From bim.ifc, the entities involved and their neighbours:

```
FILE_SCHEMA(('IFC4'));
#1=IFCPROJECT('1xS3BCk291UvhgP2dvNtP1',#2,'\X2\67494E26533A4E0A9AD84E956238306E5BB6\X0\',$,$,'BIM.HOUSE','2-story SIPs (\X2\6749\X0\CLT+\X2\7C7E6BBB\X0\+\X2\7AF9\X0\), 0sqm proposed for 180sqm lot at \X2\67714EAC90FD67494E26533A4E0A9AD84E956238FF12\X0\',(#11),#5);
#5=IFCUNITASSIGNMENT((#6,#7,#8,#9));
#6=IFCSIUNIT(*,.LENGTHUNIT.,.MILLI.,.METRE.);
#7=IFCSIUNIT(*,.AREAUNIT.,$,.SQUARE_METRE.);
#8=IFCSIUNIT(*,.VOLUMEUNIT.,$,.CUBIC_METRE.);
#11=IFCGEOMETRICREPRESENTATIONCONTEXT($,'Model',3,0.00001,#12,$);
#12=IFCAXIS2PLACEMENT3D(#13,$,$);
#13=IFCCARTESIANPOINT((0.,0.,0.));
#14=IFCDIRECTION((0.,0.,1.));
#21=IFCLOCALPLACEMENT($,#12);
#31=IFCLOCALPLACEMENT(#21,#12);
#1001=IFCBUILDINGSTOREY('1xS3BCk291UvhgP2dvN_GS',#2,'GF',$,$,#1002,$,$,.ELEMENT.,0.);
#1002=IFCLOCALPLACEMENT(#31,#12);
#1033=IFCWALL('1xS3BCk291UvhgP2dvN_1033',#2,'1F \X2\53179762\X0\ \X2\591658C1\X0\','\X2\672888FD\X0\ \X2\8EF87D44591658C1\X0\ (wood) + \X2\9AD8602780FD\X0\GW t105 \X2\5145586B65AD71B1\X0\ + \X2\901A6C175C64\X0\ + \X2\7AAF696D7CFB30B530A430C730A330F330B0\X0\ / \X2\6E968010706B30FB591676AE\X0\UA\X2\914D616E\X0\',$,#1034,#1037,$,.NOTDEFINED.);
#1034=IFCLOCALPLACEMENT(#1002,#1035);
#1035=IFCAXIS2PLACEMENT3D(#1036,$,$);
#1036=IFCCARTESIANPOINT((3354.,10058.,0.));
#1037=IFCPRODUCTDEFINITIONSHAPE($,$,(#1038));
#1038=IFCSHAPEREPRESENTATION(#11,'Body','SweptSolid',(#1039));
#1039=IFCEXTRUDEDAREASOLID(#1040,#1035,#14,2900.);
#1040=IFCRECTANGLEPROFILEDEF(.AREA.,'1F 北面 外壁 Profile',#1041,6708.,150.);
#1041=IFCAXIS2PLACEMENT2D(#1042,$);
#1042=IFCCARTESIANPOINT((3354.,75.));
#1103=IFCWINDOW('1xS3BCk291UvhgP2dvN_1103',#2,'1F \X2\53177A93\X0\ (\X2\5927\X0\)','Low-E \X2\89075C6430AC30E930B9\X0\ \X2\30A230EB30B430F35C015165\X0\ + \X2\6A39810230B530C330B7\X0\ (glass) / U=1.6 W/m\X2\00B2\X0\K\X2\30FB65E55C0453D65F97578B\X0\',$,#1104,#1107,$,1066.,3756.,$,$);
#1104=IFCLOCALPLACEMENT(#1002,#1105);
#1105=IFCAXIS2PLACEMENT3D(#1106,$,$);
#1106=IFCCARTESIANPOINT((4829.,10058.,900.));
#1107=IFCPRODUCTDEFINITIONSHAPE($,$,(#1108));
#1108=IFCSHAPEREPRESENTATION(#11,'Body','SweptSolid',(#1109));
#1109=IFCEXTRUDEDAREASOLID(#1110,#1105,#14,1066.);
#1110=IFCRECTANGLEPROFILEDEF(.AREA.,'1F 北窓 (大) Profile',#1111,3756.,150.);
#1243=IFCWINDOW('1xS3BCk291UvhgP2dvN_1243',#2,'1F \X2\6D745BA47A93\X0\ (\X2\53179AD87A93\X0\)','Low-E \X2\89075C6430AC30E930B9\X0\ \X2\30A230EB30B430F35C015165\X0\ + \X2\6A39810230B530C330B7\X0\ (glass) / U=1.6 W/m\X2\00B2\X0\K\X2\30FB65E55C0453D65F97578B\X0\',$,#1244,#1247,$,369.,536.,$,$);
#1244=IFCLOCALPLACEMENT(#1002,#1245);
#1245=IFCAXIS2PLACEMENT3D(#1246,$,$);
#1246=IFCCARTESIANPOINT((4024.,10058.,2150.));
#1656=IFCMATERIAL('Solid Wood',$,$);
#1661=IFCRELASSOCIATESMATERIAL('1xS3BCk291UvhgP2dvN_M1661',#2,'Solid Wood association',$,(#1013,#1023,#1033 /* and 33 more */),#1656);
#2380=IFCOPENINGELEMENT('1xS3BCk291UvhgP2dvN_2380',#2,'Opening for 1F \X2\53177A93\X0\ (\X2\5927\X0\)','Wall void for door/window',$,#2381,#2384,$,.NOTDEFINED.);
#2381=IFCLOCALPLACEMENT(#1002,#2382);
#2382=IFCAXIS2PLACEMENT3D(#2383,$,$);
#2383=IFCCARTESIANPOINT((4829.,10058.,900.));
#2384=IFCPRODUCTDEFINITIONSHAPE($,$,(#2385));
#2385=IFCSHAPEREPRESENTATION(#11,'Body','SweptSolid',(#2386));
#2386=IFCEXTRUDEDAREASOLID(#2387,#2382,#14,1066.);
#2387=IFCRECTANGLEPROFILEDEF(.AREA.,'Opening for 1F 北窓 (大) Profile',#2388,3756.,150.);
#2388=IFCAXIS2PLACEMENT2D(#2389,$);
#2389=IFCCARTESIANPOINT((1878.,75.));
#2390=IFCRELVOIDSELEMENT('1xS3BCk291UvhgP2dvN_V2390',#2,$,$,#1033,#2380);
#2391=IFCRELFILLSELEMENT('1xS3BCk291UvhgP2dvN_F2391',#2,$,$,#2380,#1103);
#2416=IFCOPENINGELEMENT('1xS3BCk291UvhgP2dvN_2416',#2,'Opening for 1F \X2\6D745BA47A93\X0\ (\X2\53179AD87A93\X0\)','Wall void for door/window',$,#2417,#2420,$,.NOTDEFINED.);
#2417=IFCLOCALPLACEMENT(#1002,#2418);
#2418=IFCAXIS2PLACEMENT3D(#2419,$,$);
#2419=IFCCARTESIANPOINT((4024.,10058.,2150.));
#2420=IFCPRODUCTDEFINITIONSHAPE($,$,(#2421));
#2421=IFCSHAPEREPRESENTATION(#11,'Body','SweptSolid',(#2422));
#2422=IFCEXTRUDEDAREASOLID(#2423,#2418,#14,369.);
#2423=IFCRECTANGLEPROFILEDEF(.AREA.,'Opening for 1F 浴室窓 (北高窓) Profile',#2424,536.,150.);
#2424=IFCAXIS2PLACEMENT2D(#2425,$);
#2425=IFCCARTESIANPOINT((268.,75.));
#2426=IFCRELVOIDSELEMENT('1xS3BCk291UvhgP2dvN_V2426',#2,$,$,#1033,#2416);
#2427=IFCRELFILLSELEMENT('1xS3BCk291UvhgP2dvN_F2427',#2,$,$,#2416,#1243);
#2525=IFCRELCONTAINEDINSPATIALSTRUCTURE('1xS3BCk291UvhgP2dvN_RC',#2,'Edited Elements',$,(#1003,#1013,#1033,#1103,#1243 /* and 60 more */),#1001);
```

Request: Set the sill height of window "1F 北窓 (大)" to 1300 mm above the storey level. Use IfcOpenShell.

```python
import numpy as np
import ifcopenshell
import ifcopenshell.api.geometry
import ifcopenshell.geom
import ifcopenshell.util.element
import ifcopenshell.util.placement
import ifcopenshell.util.shape
import ifcopenshell.util.unit

model = ifcopenshell.open("bim.ifc")
unit_scale = ifcopenshell.util.unit.calculate_unit_scale(model)

window = model.by_guid("1xS3BCk291UvhgP2dvN_1103")
opening = window.FillsVoids[0].RelatingOpeningElement
storey = ifcopenshell.util.element.get_container(window, ifc_class="IfcBuildingStorey")
level = ifcopenshell.util.placement.get_local_placement(storey.ObjectPlacement)[2, 3]

# The opening's origin need not be at the sill, so measure its lowest point.
shape = ifcopenshell.geom.create_shape(ifcopenshell.geom.settings(), opening)
bottom = ifcopenshell.util.shape.get_shape_bottom_elevation(shape, shape.geometry) / unit_scale
dz = level + 1300.0 - bottom

shift = np.array([0.0, 0.0, dz])
# The window is not placed relative to its opening, so move both.
for product in (opening, window):
    matrix = ifcopenshell.util.placement.get_local_placement(product.ObjectPlacement)
    matrix[:3, 3] += shift
    ifcopenshell.api.geometry.edit_object_placement(model, product=product, matrix=matrix, is_si=False)

print(f"moved by {dz * unit_scale:+.3f} m")

model.write("bim_edited.ifc")
```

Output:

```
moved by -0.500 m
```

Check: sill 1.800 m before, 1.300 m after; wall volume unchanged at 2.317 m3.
